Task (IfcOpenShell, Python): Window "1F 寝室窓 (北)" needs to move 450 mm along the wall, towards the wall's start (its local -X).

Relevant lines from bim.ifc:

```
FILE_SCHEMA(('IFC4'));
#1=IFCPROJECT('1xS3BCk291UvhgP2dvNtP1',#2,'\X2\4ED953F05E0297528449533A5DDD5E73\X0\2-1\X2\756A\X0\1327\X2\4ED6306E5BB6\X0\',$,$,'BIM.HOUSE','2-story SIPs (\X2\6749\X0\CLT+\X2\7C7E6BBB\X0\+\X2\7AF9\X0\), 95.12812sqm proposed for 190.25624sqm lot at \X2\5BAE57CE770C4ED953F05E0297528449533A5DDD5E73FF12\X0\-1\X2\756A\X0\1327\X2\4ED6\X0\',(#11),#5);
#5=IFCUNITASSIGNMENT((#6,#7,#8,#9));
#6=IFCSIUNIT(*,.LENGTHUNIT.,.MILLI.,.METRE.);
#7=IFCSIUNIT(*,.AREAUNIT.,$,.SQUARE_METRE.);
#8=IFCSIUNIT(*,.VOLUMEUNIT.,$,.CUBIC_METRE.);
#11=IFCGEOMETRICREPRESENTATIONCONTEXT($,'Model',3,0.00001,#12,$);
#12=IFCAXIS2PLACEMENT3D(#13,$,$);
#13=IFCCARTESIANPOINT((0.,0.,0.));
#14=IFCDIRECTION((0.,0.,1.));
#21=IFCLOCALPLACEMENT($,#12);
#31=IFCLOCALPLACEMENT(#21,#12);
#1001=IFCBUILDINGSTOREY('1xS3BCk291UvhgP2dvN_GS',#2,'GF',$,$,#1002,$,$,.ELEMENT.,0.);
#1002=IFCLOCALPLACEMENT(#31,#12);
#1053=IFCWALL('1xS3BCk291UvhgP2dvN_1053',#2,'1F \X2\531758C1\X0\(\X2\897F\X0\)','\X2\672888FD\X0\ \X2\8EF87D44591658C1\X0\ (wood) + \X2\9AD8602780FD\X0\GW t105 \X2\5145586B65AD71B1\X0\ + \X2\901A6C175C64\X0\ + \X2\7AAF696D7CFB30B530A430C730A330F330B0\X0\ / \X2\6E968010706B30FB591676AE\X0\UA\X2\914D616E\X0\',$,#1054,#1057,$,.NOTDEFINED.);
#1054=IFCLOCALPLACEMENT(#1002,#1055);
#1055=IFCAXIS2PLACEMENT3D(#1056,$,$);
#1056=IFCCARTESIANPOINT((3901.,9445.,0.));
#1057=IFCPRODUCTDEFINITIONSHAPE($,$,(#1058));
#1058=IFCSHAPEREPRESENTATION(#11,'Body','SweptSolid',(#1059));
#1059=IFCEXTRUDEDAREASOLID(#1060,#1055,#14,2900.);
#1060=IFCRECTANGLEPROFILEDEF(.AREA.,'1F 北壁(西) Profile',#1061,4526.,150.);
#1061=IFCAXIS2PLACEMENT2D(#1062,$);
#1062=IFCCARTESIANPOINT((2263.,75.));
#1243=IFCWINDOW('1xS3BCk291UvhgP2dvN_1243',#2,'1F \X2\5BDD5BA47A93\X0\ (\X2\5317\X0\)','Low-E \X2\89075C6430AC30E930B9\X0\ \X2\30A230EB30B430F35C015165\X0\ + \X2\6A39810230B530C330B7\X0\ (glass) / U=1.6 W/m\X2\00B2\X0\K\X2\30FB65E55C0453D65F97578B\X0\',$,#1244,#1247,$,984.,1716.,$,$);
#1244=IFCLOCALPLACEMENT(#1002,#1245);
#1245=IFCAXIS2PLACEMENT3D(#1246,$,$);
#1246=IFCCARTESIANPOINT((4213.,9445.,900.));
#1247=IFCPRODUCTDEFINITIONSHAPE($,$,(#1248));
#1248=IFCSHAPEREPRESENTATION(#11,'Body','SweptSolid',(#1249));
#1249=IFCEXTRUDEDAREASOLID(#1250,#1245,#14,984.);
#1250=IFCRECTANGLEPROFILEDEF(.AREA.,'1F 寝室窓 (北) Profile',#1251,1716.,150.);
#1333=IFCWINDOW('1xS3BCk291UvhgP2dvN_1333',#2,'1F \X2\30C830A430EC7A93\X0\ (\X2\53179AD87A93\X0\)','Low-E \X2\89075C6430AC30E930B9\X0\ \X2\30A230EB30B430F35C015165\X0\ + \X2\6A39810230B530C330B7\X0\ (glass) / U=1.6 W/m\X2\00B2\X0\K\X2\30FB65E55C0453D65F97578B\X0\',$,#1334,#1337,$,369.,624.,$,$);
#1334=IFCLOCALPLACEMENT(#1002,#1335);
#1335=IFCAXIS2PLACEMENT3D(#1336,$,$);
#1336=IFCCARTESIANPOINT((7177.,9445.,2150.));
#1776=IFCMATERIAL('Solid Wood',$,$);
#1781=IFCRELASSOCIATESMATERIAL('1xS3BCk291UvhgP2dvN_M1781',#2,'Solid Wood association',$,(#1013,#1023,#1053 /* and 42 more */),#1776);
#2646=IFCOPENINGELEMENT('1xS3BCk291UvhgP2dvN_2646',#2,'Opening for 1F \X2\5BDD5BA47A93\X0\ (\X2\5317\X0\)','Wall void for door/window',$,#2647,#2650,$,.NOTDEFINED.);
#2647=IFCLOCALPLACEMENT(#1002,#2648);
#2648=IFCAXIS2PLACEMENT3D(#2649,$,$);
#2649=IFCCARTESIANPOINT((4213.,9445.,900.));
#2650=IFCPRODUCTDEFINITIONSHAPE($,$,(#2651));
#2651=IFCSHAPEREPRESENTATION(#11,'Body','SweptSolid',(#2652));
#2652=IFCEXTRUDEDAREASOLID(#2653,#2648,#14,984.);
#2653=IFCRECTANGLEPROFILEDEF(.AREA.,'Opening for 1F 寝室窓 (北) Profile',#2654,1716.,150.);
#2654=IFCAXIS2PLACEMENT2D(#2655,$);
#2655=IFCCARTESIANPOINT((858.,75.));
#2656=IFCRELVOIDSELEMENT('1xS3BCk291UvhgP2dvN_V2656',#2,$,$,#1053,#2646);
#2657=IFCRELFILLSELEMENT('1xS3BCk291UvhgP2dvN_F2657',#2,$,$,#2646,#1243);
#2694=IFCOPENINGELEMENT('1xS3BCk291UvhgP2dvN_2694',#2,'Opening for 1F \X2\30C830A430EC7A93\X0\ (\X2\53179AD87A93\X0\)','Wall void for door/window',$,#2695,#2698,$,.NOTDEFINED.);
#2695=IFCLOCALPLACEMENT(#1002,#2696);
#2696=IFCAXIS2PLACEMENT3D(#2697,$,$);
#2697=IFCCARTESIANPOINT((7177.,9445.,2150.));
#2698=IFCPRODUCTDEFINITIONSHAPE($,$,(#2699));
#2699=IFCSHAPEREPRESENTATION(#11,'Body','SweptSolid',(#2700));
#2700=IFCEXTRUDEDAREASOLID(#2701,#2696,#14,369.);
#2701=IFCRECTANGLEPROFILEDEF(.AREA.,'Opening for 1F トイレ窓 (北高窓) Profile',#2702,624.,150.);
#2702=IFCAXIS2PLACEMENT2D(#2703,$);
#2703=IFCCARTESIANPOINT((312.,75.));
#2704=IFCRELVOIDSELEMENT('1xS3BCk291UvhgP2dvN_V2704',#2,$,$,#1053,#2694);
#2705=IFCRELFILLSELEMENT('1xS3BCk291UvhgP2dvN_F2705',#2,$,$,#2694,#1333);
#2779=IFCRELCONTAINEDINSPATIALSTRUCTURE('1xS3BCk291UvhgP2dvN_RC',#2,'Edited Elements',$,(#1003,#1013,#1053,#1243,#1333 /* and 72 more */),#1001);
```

```python
import ifcopenshell
import ifcopenshell.api.geometry
import ifcopenshell.util.placement

model = ifcopenshell.open("bim.ifc")

window = model.by_guid("1xS3BCk291UvhgP2dvN_1243")
opening = window.FillsVoids[0].RelatingOpeningElement
wall = opening.VoidsElements[0].RelatingBuildingElement

wall_matrix = ifcopenshell.util.placement.get_local_placement(wall.ObjectPlacement)
shift = wall_matrix[:3, 0] * -450.0
before = ifcopenshell.util.placement.get_local_placement(window.ObjectPlacement)[:3, 3].copy()

# The window is not placed relative to its opening, so move both.
for product in (opening, window):
    matrix = ifcopenshell.util.placement.get_local_placement(product.ObjectPlacement)
    matrix[:3, 3] += shift
    ifcopenshell.api.geometry.edit_object_placement(model, product=product, matrix=matrix, is_si=False)

after = ifcopenshell.util.placement.get_local_placement(window.ObjectPlacement)[:3, 3]
print("window moved by", (after - before).round(3) + 0.0)

model.write("bim_updated.ifc")
```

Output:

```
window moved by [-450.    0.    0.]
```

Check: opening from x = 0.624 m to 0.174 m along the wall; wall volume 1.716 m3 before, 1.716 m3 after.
